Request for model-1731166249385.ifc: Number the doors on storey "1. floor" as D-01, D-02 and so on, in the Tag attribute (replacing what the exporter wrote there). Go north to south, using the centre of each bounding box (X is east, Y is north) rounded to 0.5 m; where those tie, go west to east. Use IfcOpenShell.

First a look at what the model holds.

```python
import ifcopenshell
import ifcopenshell.util.element
import ifcopenshell.util.placement

model = ifcopenshell.open("model-1731166249385.ifc")
print(model.schema)
storey = next(s for s in model.by_type("IfcBuildingStorey") if s.Name == "1. floor")
doors = [e for e in ifcopenshell.util.element.get_decomposition(storey) if e.is_a("IfcDoor")]
for e in sorted(doors, key=lambda e: e.id()):
    origin = ifcopenshell.util.placement.get_local_placement(e.ObjectPlacement)[:3, 3]
    print(e.id(), e.Tag, e.Name, origin.round(2) + 0.0, sep=" | ")
```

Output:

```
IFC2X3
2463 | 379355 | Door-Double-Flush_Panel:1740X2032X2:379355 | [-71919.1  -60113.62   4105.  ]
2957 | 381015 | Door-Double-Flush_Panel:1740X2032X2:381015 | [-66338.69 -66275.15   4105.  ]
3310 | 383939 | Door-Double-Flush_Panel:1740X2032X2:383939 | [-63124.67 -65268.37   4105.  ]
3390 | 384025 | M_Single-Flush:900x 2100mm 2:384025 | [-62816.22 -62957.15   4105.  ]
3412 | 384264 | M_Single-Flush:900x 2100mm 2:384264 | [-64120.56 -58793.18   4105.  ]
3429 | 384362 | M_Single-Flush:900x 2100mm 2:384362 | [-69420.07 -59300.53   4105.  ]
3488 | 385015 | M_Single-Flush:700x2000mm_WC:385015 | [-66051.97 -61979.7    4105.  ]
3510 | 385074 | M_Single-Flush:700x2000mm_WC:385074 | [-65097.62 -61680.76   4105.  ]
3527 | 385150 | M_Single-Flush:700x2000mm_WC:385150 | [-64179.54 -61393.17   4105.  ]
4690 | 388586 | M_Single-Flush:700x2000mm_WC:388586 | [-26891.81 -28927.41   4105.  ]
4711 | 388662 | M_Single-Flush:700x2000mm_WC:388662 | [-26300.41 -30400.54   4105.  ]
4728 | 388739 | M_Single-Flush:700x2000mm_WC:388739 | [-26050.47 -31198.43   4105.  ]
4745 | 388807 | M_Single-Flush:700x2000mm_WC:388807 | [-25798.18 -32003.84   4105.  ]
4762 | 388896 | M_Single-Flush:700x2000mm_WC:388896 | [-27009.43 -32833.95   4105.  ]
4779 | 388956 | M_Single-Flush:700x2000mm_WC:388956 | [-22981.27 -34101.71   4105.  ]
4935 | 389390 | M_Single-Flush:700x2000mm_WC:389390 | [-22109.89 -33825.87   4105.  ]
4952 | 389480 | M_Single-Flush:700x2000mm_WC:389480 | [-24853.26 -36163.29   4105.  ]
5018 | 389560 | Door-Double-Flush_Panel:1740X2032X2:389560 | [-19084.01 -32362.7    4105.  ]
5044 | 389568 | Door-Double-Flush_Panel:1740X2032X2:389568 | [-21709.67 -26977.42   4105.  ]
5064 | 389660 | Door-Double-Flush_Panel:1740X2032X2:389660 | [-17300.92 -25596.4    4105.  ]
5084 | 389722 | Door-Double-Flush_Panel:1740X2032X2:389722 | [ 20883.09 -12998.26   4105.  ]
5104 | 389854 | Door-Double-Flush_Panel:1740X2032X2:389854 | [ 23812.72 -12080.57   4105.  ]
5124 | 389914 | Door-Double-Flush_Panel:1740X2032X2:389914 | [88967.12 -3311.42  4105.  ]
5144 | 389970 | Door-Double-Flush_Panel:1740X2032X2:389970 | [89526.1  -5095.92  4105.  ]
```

```python
import ifcopenshell
import ifcopenshell.geom
import ifcopenshell.util.element
import ifcopenshell.util.shape

model = ifcopenshell.open("model-1731166249385.ifc")
settings = ifcopenshell.geom.settings()
settings.set("use-world-coords", True)


def centre(element):
    shape = ifcopenshell.geom.create_shape(settings, element)
    return ifcopenshell.util.shape.get_bbox_centroid(shape.geometry)


storey = next(s for s in model.by_type("IfcBuildingStorey") if s.Name == "1. floor")
doors = [e for e in ifcopenshell.util.element.get_decomposition(storey) if e.is_a("IfcDoor")]

# Insertion points can sit at a corner or the storey origin, so sort by the geometry (in metres).
centres = {e: centre(e) for e in doors}
doors.sort(key=lambda e: (-round(centres[e][1] / 0.5), centres[e][0]))

for i, e in enumerate(doors, start=1):
    number = f"D-{i:02d}"
    e.Tag = number
    print(e.id(), number)

model.write("model-1731166249385-out.ifc")
```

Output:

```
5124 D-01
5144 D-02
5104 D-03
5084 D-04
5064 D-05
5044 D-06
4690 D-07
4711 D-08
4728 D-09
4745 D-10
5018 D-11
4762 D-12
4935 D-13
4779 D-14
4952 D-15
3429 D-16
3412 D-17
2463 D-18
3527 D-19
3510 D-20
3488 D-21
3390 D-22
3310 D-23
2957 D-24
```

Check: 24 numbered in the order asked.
